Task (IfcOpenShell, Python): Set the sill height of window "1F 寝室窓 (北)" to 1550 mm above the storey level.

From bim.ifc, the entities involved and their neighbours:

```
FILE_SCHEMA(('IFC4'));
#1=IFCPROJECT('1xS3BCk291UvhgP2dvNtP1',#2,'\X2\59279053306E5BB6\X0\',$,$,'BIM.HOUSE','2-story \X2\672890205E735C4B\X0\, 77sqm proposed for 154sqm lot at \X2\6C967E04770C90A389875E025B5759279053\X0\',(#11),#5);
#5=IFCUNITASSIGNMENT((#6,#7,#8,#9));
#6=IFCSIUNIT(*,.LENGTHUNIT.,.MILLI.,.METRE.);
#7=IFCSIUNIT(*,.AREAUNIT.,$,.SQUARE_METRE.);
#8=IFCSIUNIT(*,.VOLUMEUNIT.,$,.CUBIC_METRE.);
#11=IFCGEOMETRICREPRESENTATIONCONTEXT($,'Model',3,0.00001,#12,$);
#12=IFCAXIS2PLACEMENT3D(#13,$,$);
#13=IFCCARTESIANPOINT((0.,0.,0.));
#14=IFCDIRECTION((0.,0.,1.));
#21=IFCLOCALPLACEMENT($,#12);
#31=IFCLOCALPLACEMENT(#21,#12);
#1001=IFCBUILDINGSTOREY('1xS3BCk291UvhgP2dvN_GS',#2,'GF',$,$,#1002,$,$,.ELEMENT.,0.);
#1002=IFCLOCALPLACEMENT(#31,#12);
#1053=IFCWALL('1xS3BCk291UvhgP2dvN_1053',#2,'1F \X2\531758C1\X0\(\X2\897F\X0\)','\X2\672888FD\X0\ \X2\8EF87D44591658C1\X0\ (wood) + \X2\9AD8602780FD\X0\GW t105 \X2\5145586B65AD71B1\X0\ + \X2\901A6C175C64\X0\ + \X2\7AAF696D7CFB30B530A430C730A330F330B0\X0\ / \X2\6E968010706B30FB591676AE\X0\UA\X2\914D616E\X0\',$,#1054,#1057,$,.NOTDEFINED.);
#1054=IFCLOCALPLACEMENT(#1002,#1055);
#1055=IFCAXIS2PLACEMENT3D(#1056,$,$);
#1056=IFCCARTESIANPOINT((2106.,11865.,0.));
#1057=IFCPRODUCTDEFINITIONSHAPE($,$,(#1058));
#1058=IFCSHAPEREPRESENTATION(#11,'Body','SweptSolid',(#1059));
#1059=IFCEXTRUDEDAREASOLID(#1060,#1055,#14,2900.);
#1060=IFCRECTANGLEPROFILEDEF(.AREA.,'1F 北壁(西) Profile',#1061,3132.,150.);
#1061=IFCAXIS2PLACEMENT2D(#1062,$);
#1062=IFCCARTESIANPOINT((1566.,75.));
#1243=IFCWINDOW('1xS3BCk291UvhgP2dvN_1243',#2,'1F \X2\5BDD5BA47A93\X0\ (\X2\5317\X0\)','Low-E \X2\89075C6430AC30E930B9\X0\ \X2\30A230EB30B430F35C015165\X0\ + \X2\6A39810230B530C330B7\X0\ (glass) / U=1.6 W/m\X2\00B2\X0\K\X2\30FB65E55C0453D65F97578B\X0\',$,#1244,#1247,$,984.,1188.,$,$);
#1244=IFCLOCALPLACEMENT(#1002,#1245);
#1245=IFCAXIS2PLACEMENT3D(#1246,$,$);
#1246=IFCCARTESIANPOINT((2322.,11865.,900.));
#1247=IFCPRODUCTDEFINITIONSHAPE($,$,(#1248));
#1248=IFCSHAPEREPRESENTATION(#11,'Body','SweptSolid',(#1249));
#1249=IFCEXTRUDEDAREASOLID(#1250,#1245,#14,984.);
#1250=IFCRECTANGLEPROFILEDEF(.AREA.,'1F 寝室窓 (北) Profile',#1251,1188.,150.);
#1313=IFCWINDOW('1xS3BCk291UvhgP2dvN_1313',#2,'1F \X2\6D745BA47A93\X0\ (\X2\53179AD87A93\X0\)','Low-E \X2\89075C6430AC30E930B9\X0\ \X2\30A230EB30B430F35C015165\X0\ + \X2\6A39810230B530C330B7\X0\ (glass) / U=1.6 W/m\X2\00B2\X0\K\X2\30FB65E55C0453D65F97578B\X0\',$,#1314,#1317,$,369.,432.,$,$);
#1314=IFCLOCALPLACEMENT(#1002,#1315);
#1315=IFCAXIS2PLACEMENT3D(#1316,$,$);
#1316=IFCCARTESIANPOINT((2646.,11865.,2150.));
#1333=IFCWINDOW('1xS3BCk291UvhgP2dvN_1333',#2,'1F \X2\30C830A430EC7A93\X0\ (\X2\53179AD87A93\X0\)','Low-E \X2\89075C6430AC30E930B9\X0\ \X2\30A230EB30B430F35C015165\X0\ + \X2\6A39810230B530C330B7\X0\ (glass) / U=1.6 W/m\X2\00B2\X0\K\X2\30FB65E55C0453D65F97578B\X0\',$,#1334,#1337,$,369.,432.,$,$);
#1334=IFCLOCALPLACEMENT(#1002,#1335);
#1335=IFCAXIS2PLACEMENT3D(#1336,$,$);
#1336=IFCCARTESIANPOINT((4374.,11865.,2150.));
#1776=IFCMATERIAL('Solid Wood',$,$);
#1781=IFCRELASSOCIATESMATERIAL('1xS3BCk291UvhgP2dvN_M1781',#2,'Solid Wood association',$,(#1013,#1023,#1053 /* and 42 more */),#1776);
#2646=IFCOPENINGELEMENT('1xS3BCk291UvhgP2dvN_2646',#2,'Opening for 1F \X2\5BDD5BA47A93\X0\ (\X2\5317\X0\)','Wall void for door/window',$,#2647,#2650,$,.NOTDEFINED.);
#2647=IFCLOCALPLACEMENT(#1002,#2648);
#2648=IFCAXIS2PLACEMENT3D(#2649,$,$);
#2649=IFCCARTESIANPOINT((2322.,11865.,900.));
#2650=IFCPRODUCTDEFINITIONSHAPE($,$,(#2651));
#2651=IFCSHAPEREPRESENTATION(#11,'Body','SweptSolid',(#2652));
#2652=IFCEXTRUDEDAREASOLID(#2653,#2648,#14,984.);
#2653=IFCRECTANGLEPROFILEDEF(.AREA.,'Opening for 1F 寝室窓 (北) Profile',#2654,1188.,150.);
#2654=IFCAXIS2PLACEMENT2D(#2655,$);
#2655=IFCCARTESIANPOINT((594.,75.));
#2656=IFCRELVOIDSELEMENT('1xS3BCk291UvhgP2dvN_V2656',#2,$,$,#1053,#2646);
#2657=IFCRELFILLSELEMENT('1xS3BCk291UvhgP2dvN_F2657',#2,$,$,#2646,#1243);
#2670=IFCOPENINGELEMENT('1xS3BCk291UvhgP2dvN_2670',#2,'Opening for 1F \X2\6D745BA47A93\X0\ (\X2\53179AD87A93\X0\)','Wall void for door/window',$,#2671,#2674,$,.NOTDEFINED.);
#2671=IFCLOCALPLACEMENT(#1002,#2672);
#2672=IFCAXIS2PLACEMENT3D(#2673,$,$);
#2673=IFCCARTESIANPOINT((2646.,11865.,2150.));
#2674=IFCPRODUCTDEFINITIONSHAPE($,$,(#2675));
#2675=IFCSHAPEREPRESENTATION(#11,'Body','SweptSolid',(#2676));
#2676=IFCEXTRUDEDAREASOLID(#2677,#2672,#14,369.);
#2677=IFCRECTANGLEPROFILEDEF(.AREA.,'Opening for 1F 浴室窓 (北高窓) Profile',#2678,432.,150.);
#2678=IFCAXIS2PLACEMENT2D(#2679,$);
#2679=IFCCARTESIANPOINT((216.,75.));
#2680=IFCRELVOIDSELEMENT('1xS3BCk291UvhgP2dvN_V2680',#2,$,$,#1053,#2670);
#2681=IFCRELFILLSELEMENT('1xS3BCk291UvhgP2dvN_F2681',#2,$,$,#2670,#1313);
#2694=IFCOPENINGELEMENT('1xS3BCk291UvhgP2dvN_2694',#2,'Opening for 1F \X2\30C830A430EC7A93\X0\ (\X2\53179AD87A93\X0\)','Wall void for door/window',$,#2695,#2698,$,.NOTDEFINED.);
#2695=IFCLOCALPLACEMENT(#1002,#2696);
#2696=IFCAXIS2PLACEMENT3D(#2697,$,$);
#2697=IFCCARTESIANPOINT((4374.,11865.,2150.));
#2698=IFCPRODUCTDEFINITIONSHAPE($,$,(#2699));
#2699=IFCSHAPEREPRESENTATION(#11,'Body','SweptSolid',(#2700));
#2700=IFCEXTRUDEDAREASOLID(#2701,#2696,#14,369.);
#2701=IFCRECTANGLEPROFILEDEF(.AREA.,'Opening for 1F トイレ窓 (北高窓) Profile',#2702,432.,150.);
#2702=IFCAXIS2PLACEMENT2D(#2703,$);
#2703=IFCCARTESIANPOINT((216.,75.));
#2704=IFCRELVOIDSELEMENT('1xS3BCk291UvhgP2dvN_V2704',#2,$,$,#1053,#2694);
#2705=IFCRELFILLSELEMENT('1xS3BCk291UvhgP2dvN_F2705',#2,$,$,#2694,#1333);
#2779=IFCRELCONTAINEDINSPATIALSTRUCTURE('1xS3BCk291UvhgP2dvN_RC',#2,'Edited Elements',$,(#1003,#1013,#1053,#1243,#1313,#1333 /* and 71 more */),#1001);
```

```python
import numpy as np
import ifcopenshell
import ifcopenshell.api.geometry
import ifcopenshell.geom
import ifcopenshell.util.element
import ifcopenshell.util.placement
import ifcopenshell.util.shape
import ifcopenshell.util.unit

model = ifcopenshell.open("bim.ifc")
unit_scale = ifcopenshell.util.unit.calculate_unit_scale(model)

window = model.by_guid("1xS3BCk291UvhgP2dvN_1243")
opening = window.FillsVoids[0].RelatingOpeningElement
storey = ifcopenshell.util.element.get_container(window, ifc_class="IfcBuildingStorey")
level = ifcopenshell.util.placement.get_local_placement(storey.ObjectPlacement)[2, 3]

# The opening's origin need not be at the sill, so measure its lowest point.
shape = ifcopenshell.geom.create_shape(ifcopenshell.geom.settings(), opening)
bottom = ifcopenshell.util.shape.get_shape_bottom_elevation(shape, shape.geometry) / unit_scale
dz = level + 1.55 / unit_scale - bottom

shift = np.array([0.0, 0.0, dz])
# The window is not placed relative to its opening, so move both.
for product in (opening, window):
    matrix = ifcopenshell.util.placement.get_local_placement(product.ObjectPlacement)
    matrix[:3, 3] += shift
    ifcopenshell.api.geometry.edit_object_placement(model, product=product, matrix=matrix, is_si=False)

print(f"moved by {dz * unit_scale:+.3f} m")

model.write("bim_rev.ifc")
```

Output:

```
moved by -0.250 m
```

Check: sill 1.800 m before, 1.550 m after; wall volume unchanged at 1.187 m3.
